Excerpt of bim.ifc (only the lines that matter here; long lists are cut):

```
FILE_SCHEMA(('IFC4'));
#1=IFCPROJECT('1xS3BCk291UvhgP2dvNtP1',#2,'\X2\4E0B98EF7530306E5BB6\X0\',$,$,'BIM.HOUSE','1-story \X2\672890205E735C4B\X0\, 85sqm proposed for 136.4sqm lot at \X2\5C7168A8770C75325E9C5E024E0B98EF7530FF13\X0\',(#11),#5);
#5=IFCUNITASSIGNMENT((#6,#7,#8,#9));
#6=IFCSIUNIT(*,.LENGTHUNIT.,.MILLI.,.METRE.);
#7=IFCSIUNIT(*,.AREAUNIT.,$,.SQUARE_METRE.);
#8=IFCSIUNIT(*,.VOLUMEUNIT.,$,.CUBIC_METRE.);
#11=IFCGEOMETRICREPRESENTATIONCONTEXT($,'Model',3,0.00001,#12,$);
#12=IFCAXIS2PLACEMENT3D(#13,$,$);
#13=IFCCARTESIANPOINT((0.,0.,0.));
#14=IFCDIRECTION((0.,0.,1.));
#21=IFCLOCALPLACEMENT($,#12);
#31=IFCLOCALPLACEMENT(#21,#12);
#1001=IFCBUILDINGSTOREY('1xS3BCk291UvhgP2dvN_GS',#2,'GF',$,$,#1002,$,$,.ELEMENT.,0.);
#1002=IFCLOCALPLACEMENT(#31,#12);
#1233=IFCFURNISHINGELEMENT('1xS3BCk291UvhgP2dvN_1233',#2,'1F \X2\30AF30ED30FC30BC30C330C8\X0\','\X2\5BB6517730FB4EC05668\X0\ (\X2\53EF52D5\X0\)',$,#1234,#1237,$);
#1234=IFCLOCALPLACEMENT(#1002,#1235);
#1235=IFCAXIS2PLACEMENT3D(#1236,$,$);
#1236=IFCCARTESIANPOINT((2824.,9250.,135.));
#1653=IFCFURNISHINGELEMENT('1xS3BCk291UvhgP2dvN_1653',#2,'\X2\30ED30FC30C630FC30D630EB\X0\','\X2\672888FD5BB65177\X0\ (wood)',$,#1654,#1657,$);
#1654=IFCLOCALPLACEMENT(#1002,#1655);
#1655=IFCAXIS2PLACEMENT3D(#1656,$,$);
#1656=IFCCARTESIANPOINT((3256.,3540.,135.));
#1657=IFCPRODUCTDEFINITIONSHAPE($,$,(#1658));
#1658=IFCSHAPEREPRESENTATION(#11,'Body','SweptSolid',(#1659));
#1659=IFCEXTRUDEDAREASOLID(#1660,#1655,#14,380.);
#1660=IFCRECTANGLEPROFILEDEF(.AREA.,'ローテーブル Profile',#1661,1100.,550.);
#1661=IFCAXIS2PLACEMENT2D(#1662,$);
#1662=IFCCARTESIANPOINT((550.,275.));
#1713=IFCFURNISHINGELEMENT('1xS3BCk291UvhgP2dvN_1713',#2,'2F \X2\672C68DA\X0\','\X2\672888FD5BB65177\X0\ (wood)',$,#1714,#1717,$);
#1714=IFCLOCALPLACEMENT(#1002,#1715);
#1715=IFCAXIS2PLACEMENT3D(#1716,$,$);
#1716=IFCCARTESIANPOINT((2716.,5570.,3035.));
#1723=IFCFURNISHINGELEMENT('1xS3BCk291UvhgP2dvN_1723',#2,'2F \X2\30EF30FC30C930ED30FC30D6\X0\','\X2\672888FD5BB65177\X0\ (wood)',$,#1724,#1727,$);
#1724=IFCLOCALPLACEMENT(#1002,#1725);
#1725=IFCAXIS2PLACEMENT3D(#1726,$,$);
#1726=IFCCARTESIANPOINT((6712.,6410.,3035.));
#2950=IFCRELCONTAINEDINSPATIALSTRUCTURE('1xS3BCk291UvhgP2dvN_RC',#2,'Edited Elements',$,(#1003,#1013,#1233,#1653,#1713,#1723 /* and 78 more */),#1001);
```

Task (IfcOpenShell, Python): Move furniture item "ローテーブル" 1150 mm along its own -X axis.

```python
import ifcopenshell
import ifcopenshell.api.geometry
import ifcopenshell.util.placement

model = ifcopenshell.open("bim.ifc")

item = model.by_id(1653)
matrix = ifcopenshell.util.placement.get_local_placement(item.ObjectPlacement)
matrix[:3, 3] -= matrix[:3, 0] * 1150.0
ifcopenshell.api.geometry.edit_object_placement(model, product=item, matrix=matrix, is_si=False)

print(ifcopenshell.util.placement.get_local_placement(item.ObjectPlacement).round(3) + 0.0)

model.write("bim_rev.ifc")
```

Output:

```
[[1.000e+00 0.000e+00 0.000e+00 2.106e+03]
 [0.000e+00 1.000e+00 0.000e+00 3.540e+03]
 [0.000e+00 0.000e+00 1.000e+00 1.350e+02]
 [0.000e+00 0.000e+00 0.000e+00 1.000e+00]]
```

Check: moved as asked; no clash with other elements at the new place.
